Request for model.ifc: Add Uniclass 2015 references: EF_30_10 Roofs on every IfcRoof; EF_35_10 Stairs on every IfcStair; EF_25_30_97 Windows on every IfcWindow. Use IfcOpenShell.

First a look at what the model holds.

```python
import ifcopenshell

model = ifcopenshell.open("model.ifc")
print(model.schema)
print("classifications:", [c.Name for c in model.by_type("IfcClassification")])
for ifc_class in ("IfcDoor", "IfcRoof", "IfcStair", "IfcWall", "IfcWindow"):
    print(ifc_class, len(model.by_type(ifc_class)))
```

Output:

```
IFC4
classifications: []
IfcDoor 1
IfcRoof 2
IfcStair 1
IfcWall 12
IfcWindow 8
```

```python
import ifcopenshell
import ifcopenshell.api.classification

model = ifcopenshell.open("model.ifc")

system = ifcopenshell.api.classification.add_classification(model, classification="Uniclass 2015")

codes = {
    "IfcRoof": ("EF_30_10", "Roofs"),
    "IfcStair": ("EF_35_10", "Stairs"),
    "IfcWindow": ("EF_25_30_97", "Windows"),
}
for ifc_class, (code, name) in codes.items():
    products = model.by_type(ifc_class)
    ifcopenshell.api.classification.add_reference(
        model, products=products, classification=system, identification=code, name=name
    )
    print(code, len(products))

model.write("model_updated.ifc")
```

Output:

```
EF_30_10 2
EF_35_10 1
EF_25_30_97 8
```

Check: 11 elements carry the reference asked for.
